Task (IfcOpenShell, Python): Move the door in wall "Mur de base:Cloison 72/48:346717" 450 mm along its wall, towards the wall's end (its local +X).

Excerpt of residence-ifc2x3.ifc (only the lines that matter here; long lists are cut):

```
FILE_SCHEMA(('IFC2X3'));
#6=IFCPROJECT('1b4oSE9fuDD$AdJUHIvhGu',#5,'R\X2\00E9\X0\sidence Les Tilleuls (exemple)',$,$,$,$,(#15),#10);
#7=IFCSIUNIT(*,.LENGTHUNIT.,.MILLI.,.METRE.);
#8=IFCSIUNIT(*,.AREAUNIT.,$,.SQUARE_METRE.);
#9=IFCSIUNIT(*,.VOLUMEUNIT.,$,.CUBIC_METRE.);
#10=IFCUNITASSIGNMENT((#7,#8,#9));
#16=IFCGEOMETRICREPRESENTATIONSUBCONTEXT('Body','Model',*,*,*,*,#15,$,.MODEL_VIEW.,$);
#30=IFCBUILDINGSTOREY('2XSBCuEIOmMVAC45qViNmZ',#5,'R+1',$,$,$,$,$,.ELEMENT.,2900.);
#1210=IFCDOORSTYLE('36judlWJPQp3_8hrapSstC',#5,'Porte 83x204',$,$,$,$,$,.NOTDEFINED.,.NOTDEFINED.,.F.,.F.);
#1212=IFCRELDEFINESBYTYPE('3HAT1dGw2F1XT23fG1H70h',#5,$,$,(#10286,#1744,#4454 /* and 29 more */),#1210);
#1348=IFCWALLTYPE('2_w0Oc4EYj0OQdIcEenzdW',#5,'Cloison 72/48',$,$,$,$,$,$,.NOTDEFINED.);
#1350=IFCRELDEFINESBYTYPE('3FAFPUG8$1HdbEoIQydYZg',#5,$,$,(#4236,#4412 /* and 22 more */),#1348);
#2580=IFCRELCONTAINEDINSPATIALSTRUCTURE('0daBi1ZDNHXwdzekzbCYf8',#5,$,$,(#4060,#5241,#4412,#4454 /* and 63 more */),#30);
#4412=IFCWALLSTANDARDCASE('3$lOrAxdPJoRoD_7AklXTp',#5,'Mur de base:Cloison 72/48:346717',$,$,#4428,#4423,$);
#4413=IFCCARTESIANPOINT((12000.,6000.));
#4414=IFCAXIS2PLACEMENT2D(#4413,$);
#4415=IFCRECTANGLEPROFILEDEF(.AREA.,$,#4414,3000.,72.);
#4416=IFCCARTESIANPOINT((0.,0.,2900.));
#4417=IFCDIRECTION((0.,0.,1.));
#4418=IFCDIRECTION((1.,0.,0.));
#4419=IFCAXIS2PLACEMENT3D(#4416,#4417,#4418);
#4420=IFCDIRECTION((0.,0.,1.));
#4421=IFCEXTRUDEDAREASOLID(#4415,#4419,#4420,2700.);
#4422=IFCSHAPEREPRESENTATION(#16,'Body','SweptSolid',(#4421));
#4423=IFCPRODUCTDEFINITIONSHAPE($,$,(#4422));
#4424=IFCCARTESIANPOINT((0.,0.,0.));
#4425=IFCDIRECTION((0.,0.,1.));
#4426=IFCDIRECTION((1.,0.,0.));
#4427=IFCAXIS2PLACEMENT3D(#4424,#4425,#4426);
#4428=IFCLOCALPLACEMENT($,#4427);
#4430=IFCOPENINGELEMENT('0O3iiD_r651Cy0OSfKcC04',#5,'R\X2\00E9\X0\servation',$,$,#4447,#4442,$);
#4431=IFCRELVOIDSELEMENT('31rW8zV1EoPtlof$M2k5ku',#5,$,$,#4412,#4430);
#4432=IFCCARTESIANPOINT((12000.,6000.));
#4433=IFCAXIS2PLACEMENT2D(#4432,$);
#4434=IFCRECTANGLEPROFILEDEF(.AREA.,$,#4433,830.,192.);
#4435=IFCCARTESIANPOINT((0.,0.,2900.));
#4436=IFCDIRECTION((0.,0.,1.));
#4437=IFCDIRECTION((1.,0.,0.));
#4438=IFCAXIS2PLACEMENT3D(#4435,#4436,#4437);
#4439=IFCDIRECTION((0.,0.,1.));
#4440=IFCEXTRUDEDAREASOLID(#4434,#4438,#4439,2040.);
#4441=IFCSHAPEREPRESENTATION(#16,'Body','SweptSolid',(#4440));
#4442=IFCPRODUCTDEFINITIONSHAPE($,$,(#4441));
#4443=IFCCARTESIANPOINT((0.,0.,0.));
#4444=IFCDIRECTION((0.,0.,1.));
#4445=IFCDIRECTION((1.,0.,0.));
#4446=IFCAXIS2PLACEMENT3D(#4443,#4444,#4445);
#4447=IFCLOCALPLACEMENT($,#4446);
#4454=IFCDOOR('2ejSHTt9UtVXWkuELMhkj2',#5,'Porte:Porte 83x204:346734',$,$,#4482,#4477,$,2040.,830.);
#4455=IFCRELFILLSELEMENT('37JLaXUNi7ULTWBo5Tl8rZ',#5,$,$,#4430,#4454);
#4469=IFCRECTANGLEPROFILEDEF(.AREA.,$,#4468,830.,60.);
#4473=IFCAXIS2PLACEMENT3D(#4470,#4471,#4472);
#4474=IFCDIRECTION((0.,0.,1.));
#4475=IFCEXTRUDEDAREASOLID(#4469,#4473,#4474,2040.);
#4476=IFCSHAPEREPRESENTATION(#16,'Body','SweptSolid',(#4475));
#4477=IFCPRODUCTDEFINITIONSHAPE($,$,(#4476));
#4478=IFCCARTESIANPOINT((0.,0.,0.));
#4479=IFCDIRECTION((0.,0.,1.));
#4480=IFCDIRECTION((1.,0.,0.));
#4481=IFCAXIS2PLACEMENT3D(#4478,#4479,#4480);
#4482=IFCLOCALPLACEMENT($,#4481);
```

```python
import ifcopenshell
import ifcopenshell.api.geometry
import ifcopenshell.util.placement
import ifcopenshell.util.unit

model = ifcopenshell.open("residence-ifc2x3.ifc")
unit_scale = ifcopenshell.util.unit.calculate_unit_scale(model)

door = model.by_guid("2ejSHTt9UtVXWkuELMhkj2")
opening = door.FillsVoids[0].RelatingOpeningElement
wall = opening.VoidsElements[0].RelatingBuildingElement

wall_matrix = ifcopenshell.util.placement.get_local_placement(wall.ObjectPlacement)
shift = wall_matrix[:3, 0] * 0.45 / unit_scale
before = ifcopenshell.util.placement.get_local_placement(door.ObjectPlacement)[:3, 3].copy()

# The door is not placed relative to its opening, so move both.
for product in (opening, door):
    matrix = ifcopenshell.util.placement.get_local_placement(product.ObjectPlacement)
    matrix[:3, 3] += shift
    ifcopenshell.api.geometry.edit_object_placement(model, product=product, matrix=matrix, is_si=False)

after = ifcopenshell.util.placement.get_local_placement(door.ObjectPlacement)[:3, 3]
print("door moved by", (after - before).round(3) + 0.0)

model.write("residence-ifc2x3_edited.ifc")
```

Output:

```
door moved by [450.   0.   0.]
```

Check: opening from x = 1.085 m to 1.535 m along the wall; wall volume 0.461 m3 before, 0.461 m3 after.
